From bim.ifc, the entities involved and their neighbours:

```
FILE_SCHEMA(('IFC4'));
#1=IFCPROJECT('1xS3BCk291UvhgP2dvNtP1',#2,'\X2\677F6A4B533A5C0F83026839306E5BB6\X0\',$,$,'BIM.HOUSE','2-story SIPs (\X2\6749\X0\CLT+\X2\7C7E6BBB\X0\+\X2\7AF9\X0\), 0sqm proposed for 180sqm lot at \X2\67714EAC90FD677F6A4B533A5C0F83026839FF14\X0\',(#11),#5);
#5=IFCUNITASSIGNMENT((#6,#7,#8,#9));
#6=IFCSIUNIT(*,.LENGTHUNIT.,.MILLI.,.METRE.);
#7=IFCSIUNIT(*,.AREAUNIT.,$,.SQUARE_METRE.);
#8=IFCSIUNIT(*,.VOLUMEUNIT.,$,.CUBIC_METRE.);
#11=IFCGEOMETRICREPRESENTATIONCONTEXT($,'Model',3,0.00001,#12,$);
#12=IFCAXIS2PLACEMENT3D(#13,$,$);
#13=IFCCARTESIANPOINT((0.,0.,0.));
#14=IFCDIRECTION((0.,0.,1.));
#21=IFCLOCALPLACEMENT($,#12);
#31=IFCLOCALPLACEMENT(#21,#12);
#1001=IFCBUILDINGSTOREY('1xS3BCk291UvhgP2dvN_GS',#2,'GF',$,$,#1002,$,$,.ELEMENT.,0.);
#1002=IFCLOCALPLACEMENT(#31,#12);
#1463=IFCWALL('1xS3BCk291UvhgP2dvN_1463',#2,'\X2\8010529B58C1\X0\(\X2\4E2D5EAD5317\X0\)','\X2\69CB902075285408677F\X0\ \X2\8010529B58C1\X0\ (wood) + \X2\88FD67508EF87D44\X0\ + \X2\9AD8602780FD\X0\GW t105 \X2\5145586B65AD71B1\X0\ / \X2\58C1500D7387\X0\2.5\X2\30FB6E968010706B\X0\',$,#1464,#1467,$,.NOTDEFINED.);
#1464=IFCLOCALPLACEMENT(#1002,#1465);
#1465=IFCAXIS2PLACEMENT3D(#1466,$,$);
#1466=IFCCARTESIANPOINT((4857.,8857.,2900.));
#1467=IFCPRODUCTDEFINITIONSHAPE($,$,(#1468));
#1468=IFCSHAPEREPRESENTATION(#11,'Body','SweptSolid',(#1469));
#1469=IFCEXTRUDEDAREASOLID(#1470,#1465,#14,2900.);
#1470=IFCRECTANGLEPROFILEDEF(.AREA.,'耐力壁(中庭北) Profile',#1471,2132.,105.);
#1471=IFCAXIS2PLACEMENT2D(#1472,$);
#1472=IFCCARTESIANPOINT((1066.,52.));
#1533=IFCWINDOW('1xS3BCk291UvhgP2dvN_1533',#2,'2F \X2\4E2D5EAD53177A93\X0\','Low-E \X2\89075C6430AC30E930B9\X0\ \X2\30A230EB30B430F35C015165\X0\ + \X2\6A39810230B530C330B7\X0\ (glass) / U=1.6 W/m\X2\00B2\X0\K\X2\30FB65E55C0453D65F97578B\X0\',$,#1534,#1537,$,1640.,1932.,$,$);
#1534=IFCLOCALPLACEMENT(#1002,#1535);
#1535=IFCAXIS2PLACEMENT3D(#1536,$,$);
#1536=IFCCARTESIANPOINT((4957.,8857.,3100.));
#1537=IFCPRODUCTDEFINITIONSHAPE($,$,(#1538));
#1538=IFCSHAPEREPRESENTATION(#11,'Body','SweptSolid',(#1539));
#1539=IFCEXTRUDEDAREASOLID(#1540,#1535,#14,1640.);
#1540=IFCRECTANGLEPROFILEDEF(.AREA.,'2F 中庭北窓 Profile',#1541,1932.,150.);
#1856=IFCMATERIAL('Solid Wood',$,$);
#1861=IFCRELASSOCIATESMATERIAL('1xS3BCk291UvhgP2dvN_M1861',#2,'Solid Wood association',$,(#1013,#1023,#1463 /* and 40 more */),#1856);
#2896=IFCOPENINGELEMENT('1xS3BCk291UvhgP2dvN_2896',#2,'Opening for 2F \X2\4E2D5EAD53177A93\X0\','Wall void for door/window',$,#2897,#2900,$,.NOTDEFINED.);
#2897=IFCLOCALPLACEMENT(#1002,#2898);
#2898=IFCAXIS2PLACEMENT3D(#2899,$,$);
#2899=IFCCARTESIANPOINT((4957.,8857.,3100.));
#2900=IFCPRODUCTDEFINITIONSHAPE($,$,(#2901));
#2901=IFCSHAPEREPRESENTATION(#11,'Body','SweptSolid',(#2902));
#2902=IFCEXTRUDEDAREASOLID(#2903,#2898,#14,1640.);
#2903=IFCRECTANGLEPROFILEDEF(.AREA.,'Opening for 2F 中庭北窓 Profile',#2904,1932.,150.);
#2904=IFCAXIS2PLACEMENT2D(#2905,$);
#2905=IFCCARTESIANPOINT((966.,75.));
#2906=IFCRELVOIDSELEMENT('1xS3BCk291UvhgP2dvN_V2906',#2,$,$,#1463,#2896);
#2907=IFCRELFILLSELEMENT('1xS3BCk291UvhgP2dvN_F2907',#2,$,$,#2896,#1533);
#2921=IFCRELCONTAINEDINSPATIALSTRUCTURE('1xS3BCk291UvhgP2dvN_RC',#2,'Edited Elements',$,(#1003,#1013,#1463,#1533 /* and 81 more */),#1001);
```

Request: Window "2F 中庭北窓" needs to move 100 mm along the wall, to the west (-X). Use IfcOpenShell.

```python
import ifcopenshell
import ifcopenshell.api.geometry
import ifcopenshell.util.placement
import ifcopenshell.util.unit

model = ifcopenshell.open("bim.ifc")
unit_scale = ifcopenshell.util.unit.calculate_unit_scale(model)

window = model.by_guid("1xS3BCk291UvhgP2dvN_1533")
opening = window.FillsVoids[0].RelatingOpeningElement
wall = opening.VoidsElements[0].RelatingBuildingElement

wall_matrix = ifcopenshell.util.placement.get_local_placement(wall.ObjectPlacement)
shift = wall_matrix[:3, 0] * -0.1 / unit_scale
before = ifcopenshell.util.placement.get_local_placement(window.ObjectPlacement)[:3, 3].copy()

# The window is not placed relative to its opening, so move both.
for product in (opening, window):
    matrix = ifcopenshell.util.placement.get_local_placement(product.ObjectPlacement)
    matrix[:3, 3] += shift
    ifcopenshell.api.geometry.edit_object_placement(model, product=product, matrix=matrix, is_si=False)

after = ifcopenshell.util.placement.get_local_placement(window.ObjectPlacement)[:3, 3]
print("window moved by", (after - before).round(3) + 0.0)

model.write("bim_rev.ifc")
```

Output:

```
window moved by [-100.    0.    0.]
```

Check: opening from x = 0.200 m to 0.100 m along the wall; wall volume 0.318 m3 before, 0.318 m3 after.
